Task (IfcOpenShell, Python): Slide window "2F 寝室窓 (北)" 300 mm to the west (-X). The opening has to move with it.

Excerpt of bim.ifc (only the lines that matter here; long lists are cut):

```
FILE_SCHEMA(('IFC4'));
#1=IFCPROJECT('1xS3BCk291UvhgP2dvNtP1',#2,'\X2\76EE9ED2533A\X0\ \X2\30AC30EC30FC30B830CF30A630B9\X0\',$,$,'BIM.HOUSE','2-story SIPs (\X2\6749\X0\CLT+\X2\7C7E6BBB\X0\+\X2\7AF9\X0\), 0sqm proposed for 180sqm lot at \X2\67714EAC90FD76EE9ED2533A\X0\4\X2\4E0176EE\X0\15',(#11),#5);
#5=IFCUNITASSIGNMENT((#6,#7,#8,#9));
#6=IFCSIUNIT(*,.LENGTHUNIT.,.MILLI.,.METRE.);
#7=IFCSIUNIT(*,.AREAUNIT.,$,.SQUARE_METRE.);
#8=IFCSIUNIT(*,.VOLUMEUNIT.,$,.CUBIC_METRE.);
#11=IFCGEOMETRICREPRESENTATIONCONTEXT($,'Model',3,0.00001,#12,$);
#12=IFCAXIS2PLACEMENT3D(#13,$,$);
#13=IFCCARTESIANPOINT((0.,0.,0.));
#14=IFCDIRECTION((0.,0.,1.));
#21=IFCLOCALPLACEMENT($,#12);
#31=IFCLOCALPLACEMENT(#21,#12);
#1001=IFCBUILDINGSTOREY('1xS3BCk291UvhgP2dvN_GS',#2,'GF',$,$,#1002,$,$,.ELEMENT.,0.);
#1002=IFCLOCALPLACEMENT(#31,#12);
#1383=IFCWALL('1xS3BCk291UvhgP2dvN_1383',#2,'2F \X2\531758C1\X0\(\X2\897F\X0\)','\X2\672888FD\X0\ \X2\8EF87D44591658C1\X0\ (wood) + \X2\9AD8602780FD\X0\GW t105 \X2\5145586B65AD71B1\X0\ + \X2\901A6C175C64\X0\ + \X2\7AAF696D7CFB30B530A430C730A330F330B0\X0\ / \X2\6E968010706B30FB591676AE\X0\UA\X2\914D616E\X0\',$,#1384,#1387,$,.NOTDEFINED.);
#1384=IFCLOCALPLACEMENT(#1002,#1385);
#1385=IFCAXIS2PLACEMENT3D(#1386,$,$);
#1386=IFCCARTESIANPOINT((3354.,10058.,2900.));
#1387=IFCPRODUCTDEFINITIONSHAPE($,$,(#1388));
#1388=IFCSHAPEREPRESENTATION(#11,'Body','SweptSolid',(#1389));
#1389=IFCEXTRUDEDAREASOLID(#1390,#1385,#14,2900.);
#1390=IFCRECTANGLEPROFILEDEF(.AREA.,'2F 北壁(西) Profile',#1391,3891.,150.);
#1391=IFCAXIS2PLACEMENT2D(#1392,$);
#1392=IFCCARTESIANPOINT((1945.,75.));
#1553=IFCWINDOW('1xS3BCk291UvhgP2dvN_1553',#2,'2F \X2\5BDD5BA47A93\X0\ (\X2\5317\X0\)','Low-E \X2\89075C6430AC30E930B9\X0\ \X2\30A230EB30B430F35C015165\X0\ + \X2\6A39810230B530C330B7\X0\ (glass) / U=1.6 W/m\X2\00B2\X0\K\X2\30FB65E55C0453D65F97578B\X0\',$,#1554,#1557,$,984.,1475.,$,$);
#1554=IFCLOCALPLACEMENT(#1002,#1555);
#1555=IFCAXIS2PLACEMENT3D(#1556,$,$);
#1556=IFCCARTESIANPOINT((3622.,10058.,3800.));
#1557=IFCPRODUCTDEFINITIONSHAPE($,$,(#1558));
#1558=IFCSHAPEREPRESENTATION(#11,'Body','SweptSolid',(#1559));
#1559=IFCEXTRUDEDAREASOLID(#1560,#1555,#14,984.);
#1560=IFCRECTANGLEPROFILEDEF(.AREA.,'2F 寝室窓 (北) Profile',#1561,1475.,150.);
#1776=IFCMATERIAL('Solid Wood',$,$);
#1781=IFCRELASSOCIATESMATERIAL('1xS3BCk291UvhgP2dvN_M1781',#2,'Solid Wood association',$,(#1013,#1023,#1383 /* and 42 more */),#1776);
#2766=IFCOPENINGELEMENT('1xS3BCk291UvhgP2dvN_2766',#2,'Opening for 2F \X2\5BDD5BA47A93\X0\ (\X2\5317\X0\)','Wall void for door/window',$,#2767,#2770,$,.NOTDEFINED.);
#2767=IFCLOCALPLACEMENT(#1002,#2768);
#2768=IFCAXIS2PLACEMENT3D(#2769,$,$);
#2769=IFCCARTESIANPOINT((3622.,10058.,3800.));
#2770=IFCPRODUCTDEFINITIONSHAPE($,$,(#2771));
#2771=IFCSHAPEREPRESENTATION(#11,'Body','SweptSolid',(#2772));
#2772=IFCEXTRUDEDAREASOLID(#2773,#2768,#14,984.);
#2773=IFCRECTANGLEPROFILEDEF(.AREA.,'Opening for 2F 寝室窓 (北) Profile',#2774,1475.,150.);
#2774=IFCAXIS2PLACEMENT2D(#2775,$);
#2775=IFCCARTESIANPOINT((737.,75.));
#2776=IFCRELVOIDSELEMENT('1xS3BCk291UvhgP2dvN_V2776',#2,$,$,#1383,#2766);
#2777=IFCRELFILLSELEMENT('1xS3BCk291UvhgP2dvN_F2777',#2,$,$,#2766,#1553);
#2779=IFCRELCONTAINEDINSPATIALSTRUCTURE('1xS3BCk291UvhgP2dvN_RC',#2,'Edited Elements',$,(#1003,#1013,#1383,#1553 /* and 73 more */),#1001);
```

```python
import ifcopenshell
import ifcopenshell.api.geometry
import ifcopenshell.util.placement

model = ifcopenshell.open("bim.ifc")

window = model.by_guid("1xS3BCk291UvhgP2dvN_1553")
opening = window.FillsVoids[0].RelatingOpeningElement
wall = opening.VoidsElements[0].RelatingBuildingElement

wall_matrix = ifcopenshell.util.placement.get_local_placement(wall.ObjectPlacement)
shift = wall_matrix[:3, 0] * -300.0
before = ifcopenshell.util.placement.get_local_placement(window.ObjectPlacement)[:3, 3].copy()

# The window is not placed relative to its opening, so move both.
for product in (opening, window):
    matrix = ifcopenshell.util.placement.get_local_placement(product.ObjectPlacement)
    matrix[:3, 3] += shift
    ifcopenshell.api.geometry.edit_object_placement(model, product=product, matrix=matrix, is_si=False)

after = ifcopenshell.util.placement.get_local_placement(window.ObjectPlacement)[:3, 3]
print("window moved by", (after - before).round(3) + 0.0)

model.write("bim-out.ifc")
```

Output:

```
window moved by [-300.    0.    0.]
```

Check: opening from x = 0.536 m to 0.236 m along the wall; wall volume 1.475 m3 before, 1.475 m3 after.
